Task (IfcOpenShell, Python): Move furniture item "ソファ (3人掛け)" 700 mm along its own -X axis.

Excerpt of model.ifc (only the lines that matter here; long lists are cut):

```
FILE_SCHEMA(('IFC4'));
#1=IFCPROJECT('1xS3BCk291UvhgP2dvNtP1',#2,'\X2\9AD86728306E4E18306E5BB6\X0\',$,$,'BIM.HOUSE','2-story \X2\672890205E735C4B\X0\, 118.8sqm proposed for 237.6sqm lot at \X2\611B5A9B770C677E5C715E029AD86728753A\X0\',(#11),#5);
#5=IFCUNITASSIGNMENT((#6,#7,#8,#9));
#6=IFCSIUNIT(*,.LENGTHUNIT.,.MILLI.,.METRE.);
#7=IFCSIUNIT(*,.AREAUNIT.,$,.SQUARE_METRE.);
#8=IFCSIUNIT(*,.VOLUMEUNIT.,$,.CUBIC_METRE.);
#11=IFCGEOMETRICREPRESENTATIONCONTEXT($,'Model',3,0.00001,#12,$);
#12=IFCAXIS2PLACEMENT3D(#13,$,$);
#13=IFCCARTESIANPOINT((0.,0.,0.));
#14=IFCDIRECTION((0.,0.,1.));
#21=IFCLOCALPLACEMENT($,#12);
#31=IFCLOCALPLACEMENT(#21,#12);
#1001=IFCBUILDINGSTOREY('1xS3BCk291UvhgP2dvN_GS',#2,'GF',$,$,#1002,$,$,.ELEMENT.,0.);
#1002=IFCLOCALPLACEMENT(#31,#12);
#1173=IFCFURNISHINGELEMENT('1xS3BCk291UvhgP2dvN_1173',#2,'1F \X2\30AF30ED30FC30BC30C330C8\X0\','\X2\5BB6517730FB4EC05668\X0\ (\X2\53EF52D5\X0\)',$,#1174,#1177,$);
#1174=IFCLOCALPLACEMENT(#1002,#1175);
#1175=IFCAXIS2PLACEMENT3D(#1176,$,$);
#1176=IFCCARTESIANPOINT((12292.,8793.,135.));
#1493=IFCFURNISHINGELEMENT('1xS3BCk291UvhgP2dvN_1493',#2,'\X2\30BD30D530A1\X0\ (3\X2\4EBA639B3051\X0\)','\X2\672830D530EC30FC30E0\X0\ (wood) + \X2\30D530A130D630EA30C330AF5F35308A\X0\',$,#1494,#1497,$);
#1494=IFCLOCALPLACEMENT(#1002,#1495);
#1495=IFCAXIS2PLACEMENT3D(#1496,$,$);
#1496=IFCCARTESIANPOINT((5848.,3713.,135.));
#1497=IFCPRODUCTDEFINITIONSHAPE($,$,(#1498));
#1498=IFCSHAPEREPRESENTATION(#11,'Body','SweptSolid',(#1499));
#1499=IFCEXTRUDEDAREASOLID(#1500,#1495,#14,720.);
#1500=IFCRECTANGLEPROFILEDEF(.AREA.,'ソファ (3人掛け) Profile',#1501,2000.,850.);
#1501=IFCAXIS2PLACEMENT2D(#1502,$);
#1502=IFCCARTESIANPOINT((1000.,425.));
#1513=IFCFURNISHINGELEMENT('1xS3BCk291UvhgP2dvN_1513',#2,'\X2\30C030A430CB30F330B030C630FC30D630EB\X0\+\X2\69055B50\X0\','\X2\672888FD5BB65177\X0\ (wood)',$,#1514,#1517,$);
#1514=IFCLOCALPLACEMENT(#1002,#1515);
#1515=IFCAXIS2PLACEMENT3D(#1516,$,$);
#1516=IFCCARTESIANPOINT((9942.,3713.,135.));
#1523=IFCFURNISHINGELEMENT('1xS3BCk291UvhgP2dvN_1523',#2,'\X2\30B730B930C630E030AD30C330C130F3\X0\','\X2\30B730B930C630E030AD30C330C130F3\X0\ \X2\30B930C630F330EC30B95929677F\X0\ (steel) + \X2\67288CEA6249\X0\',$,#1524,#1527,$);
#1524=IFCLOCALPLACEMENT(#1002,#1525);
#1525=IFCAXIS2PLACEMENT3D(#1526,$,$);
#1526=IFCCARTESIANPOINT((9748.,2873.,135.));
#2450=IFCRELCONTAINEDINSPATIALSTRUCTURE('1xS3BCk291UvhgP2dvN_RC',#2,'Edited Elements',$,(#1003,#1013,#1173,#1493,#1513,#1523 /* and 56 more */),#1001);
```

```python
import ifcopenshell
import ifcopenshell.api.geometry
import ifcopenshell.util.placement
import ifcopenshell.util.unit

model = ifcopenshell.open("model.ifc")
unit_scale = ifcopenshell.util.unit.calculate_unit_scale(model)

item = model.by_guid("1xS3BCk291UvhgP2dvN_1493")
matrix = ifcopenshell.util.placement.get_local_placement(item.ObjectPlacement)
matrix[:3, 3] -= matrix[:3, 0] * 0.7 / unit_scale
ifcopenshell.api.geometry.edit_object_placement(model, product=item, matrix=matrix, is_si=False)

print(ifcopenshell.util.placement.get_local_placement(item.ObjectPlacement).round(3) + 0.0)

model.write("model_updated.ifc")
```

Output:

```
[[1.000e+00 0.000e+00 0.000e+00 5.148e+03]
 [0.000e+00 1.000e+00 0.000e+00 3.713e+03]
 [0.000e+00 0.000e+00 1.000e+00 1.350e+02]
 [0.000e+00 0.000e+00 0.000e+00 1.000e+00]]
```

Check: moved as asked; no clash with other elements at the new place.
